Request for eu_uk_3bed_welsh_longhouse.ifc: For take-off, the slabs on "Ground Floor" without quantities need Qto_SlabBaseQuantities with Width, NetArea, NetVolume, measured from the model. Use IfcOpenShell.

First a look at what the model holds.

```python
import ifcopenshell
import ifcopenshell.util.element
import ifcopenshell.util.unit

model = ifcopenshell.open("eu_uk_3bed_welsh_longhouse.ifc")
print(model.schema)
for unit_type in ("LENGTHUNIT", "AREAUNIT", "VOLUMEUNIT"):
    print(unit_type, ifcopenshell.util.unit.calculate_unit_scale(model, unit_type))
storey = next(s for s in model.by_type("IfcBuildingStorey") if s.Name == "Ground Floor")
slabs = [e for e in ifcopenshell.util.element.get_decomposition(storey) if e.is_a("IfcSlab")]
for e in sorted(slabs, key=lambda e: e.id()):
    print(e.id(), e.is_a(), e.Name, list(ifcopenshell.util.element.get_psets(e, qtos_only=True)), sep=" | ")
```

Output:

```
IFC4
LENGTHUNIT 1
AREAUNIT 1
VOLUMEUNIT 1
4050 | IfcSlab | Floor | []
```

```python
import ifcopenshell
import ifcopenshell.api.pset
import ifcopenshell.geom
import ifcopenshell.util.element
import ifcopenshell.util.shape
import ifcopenshell.util.unit

model = ifcopenshell.open("eu_uk_3bed_welsh_longhouse.ifc")
unit_scale = ifcopenshell.util.unit.calculate_unit_scale(model)
area_scale = ifcopenshell.util.unit.calculate_unit_scale(model, "AREAUNIT")
volume_scale = ifcopenshell.util.unit.calculate_unit_scale(model, "VOLUMEUNIT")
settings = ifcopenshell.geom.settings()

storey = next(s for s in model.by_type("IfcBuildingStorey") if s.Name == "Ground Floor")
slabs = [e for e in ifcopenshell.util.element.get_decomposition(storey) if e.is_a("IfcSlab")]

for e in sorted(slabs, key=lambda e: e.id()):
    if ifcopenshell.util.element.get_psets(e, qtos_only=True, should_inherit=False):
        continue
    # Geometry comes back in metres, in the element's own axes.
    shape = ifcopenshell.geom.create_shape(settings, e)
    values = {
        "Width": ifcopenshell.util.shape.get_z(shape.geometry) / unit_scale,
        "NetArea": ifcopenshell.util.shape.get_footprint_area(shape.geometry) / area_scale,
        "NetVolume": ifcopenshell.util.shape.get_volume(shape.geometry) / volume_scale,
    }
    qto = ifcopenshell.api.pset.add_qto(model, product=e, name="Qto_SlabBaseQuantities")
    ifcopenshell.api.pset.edit_qto(model, qto=qto, properties=values)
    print(e.id(), {k: round(v, 3) for k, v in values.items()})

model.write("eu_uk_3bed_welsh_longhouse_updated.ifc")
```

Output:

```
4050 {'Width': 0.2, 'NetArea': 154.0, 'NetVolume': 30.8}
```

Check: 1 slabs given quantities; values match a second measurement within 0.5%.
